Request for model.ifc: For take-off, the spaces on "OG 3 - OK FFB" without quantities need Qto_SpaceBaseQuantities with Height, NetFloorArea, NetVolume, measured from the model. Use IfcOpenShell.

First a look at what the model holds.

```python
import ifcopenshell
import ifcopenshell.util.element
import ifcopenshell.util.unit

model = ifcopenshell.open("model.ifc")
print(model.schema)
for unit_type in ("LENGTHUNIT", "AREAUNIT", "VOLUMEUNIT"):
    print(unit_type, ifcopenshell.util.unit.calculate_unit_scale(model, unit_type))
storey = next(s for s in model.by_type("IfcBuildingStorey") if s.Name == "OG 3 - OK FFB")
spaces = [e for e in ifcopenshell.util.element.get_decomposition(storey) if e.is_a("IfcSpace")]
for e in sorted(spaces, key=lambda e: e.id()):
    print(e.id(), e.is_a(), e.Name, list(ifcopenshell.util.element.get_psets(e, qtos_only=True)), sep=" | ")
```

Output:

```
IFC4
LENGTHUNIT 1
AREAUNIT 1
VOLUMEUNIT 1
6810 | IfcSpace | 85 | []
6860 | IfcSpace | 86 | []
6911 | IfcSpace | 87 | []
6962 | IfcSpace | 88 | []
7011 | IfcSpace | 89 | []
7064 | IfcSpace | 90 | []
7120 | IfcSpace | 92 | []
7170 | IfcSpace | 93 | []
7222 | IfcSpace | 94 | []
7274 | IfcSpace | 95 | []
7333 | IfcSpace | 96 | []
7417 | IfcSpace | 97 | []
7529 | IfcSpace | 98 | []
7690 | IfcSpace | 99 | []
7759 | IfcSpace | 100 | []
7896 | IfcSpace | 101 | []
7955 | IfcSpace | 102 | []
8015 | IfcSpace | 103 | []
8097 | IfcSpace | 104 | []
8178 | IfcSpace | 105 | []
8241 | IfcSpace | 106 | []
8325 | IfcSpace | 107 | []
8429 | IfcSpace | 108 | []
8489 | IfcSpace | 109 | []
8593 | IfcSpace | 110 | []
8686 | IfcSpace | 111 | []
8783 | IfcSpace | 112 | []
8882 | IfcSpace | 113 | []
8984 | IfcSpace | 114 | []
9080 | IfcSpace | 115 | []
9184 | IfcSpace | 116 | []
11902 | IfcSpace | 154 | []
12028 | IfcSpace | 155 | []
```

```python
import ifcopenshell
import ifcopenshell.api.pset
import ifcopenshell.geom
import ifcopenshell.util.element
import ifcopenshell.util.shape
import ifcopenshell.util.unit

model = ifcopenshell.open("model.ifc")
unit_scale = ifcopenshell.util.unit.calculate_unit_scale(model)
area_scale = ifcopenshell.util.unit.calculate_unit_scale(model, "AREAUNIT")
volume_scale = ifcopenshell.util.unit.calculate_unit_scale(model, "VOLUMEUNIT")
settings = ifcopenshell.geom.settings()

storey = next(s for s in model.by_type("IfcBuildingStorey") if s.Name == "OG 3 - OK FFB")
spaces = [e for e in ifcopenshell.util.element.get_decomposition(storey) if e.is_a("IfcSpace")]

for e in sorted(spaces, key=lambda e: e.id()):
    if ifcopenshell.util.element.get_psets(e, qtos_only=True, should_inherit=False):
        continue
    # Geometry comes back in metres, in the element's own axes.
    shape = ifcopenshell.geom.create_shape(settings, e)
    values = {
        "Height": ifcopenshell.util.shape.get_z(shape.geometry) / unit_scale,
        "NetFloorArea": ifcopenshell.util.shape.get_footprint_area(shape.geometry) / area_scale,
        "NetVolume": ifcopenshell.util.shape.get_volume(shape.geometry) / volume_scale,
    }
    qto = ifcopenshell.api.pset.add_qto(model, product=e, name="Qto_SpaceBaseQuantities")
    ifcopenshell.api.pset.edit_qto(model, qto=qto, properties=values)
    print(e.id(), {k: round(v, 3) for k, v in values.items()})

model.write("model_rev.ifc")
```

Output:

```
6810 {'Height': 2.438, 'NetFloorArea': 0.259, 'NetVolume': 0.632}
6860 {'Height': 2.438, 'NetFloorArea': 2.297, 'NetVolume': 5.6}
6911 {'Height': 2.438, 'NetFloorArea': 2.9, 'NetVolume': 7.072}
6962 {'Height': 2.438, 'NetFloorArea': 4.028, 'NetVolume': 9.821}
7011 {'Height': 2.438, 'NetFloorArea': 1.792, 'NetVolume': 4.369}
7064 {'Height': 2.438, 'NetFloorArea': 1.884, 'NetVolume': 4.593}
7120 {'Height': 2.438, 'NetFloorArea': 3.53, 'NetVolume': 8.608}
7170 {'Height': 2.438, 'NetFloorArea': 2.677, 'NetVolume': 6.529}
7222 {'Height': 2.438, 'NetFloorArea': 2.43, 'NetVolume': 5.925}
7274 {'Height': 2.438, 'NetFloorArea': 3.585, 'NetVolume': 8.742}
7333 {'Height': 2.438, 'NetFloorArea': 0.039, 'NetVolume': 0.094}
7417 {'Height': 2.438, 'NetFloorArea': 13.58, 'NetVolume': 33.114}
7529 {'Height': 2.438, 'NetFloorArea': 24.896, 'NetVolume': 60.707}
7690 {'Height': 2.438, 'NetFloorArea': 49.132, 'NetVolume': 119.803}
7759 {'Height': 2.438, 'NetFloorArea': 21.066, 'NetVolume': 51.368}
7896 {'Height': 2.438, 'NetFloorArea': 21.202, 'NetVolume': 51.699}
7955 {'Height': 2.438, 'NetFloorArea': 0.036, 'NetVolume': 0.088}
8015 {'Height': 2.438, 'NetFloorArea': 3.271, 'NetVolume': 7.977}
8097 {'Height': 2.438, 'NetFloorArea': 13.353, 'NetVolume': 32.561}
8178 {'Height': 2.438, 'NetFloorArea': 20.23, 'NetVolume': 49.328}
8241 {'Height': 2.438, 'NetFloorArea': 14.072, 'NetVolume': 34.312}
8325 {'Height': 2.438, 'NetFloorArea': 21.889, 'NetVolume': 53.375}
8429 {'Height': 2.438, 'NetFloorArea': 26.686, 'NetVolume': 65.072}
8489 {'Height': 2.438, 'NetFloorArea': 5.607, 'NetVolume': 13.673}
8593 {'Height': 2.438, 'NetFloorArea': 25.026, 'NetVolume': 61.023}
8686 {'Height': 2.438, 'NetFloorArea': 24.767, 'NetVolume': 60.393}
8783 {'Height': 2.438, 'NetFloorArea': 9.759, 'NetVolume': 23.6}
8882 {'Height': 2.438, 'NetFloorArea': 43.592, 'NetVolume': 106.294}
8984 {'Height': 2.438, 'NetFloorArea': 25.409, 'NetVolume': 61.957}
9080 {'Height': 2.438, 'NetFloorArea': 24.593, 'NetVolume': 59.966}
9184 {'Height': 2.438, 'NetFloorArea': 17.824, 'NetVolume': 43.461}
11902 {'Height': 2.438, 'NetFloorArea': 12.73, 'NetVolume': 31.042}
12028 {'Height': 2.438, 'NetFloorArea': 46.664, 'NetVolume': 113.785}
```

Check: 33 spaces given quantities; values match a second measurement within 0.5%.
